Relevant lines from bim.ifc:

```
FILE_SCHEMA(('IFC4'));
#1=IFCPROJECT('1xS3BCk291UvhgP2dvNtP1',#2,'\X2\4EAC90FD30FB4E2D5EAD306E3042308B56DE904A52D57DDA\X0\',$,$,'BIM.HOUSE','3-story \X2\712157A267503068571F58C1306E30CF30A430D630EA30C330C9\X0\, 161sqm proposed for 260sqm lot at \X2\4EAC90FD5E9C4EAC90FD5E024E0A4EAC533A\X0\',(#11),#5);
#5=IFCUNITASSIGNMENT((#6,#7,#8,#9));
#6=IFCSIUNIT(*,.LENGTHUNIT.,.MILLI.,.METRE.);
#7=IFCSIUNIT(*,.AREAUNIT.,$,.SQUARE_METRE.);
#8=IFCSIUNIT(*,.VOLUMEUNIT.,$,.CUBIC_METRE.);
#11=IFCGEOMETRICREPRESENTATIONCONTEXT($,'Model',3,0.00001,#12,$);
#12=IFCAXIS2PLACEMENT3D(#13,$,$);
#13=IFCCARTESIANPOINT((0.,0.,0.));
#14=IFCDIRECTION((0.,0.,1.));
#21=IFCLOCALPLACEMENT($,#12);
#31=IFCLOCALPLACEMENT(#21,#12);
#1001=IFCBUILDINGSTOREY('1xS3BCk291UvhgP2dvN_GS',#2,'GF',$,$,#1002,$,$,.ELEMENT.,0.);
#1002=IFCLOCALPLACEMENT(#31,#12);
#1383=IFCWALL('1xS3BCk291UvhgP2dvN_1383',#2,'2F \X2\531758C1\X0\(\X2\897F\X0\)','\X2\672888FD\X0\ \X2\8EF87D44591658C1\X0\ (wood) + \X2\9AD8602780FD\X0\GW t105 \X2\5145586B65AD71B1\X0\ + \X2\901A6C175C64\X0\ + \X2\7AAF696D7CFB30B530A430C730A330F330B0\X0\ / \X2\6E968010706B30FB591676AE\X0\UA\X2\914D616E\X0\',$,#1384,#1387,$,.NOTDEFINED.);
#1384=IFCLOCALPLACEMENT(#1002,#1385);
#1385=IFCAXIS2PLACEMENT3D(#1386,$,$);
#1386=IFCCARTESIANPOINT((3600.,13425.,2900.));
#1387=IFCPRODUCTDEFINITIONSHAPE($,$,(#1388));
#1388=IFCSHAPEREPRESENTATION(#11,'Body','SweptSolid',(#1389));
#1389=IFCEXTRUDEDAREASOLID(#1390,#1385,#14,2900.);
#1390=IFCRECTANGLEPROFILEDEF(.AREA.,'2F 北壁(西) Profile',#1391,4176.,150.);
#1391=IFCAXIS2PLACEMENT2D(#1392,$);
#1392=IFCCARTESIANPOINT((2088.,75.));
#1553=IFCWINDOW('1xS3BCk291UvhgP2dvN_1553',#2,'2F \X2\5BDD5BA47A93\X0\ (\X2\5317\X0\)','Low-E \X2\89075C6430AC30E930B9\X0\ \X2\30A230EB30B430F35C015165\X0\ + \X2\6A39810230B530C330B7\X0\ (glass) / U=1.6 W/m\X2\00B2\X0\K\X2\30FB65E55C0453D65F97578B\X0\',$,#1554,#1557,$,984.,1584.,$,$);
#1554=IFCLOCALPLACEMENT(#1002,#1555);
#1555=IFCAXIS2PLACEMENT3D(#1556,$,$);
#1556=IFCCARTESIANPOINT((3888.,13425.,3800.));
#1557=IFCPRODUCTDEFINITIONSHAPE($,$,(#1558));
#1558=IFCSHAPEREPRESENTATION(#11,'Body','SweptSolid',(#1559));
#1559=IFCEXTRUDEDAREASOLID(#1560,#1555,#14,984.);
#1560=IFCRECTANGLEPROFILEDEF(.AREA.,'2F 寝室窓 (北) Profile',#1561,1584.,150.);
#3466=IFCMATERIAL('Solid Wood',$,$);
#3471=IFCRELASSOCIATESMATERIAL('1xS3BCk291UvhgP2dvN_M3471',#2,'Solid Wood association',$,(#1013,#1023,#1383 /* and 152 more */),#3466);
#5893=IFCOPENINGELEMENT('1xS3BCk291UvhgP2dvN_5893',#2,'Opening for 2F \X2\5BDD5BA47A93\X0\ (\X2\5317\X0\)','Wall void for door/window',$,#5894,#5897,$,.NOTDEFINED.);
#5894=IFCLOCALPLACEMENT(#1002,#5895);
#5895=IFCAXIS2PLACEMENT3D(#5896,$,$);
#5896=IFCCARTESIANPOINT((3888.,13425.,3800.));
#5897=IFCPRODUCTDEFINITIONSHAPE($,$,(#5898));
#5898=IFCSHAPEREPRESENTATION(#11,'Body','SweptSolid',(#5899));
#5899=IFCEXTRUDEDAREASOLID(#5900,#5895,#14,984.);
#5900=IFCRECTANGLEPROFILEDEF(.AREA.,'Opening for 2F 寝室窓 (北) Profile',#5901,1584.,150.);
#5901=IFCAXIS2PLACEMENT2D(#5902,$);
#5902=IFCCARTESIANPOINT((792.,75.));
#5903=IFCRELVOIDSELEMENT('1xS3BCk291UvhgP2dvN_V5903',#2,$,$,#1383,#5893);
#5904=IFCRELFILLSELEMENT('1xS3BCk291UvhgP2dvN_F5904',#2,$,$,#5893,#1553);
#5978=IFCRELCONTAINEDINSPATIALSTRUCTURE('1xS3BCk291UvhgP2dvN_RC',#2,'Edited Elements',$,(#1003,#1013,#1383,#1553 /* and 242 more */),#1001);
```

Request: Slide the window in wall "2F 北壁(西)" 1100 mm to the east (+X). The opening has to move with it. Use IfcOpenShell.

```python
import ifcopenshell
import ifcopenshell.api.geometry
import ifcopenshell.util.placement
import ifcopenshell.util.unit

model = ifcopenshell.open("bim.ifc")
unit_scale = ifcopenshell.util.unit.calculate_unit_scale(model)

window = model.by_guid("1xS3BCk291UvhgP2dvN_1553")
opening = window.FillsVoids[0].RelatingOpeningElement
wall = opening.VoidsElements[0].RelatingBuildingElement

wall_matrix = ifcopenshell.util.placement.get_local_placement(wall.ObjectPlacement)
shift = wall_matrix[:3, 0] * 1.1 / unit_scale
before = ifcopenshell.util.placement.get_local_placement(window.ObjectPlacement)[:3, 3].copy()

# The window is not placed relative to its opening, so move both.
for product in (opening, window):
    matrix = ifcopenshell.util.placement.get_local_placement(product.ObjectPlacement)
    matrix[:3, 3] += shift
    ifcopenshell.api.geometry.edit_object_placement(model, product=product, matrix=matrix, is_si=False)

after = ifcopenshell.util.placement.get_local_placement(window.ObjectPlacement)[:3, 3]
print("window moved by", (after - before).round(3) + 0.0)

model.write("bim_edited.ifc")
```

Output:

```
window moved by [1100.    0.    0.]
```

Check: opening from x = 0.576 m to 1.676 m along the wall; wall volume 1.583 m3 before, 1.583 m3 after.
